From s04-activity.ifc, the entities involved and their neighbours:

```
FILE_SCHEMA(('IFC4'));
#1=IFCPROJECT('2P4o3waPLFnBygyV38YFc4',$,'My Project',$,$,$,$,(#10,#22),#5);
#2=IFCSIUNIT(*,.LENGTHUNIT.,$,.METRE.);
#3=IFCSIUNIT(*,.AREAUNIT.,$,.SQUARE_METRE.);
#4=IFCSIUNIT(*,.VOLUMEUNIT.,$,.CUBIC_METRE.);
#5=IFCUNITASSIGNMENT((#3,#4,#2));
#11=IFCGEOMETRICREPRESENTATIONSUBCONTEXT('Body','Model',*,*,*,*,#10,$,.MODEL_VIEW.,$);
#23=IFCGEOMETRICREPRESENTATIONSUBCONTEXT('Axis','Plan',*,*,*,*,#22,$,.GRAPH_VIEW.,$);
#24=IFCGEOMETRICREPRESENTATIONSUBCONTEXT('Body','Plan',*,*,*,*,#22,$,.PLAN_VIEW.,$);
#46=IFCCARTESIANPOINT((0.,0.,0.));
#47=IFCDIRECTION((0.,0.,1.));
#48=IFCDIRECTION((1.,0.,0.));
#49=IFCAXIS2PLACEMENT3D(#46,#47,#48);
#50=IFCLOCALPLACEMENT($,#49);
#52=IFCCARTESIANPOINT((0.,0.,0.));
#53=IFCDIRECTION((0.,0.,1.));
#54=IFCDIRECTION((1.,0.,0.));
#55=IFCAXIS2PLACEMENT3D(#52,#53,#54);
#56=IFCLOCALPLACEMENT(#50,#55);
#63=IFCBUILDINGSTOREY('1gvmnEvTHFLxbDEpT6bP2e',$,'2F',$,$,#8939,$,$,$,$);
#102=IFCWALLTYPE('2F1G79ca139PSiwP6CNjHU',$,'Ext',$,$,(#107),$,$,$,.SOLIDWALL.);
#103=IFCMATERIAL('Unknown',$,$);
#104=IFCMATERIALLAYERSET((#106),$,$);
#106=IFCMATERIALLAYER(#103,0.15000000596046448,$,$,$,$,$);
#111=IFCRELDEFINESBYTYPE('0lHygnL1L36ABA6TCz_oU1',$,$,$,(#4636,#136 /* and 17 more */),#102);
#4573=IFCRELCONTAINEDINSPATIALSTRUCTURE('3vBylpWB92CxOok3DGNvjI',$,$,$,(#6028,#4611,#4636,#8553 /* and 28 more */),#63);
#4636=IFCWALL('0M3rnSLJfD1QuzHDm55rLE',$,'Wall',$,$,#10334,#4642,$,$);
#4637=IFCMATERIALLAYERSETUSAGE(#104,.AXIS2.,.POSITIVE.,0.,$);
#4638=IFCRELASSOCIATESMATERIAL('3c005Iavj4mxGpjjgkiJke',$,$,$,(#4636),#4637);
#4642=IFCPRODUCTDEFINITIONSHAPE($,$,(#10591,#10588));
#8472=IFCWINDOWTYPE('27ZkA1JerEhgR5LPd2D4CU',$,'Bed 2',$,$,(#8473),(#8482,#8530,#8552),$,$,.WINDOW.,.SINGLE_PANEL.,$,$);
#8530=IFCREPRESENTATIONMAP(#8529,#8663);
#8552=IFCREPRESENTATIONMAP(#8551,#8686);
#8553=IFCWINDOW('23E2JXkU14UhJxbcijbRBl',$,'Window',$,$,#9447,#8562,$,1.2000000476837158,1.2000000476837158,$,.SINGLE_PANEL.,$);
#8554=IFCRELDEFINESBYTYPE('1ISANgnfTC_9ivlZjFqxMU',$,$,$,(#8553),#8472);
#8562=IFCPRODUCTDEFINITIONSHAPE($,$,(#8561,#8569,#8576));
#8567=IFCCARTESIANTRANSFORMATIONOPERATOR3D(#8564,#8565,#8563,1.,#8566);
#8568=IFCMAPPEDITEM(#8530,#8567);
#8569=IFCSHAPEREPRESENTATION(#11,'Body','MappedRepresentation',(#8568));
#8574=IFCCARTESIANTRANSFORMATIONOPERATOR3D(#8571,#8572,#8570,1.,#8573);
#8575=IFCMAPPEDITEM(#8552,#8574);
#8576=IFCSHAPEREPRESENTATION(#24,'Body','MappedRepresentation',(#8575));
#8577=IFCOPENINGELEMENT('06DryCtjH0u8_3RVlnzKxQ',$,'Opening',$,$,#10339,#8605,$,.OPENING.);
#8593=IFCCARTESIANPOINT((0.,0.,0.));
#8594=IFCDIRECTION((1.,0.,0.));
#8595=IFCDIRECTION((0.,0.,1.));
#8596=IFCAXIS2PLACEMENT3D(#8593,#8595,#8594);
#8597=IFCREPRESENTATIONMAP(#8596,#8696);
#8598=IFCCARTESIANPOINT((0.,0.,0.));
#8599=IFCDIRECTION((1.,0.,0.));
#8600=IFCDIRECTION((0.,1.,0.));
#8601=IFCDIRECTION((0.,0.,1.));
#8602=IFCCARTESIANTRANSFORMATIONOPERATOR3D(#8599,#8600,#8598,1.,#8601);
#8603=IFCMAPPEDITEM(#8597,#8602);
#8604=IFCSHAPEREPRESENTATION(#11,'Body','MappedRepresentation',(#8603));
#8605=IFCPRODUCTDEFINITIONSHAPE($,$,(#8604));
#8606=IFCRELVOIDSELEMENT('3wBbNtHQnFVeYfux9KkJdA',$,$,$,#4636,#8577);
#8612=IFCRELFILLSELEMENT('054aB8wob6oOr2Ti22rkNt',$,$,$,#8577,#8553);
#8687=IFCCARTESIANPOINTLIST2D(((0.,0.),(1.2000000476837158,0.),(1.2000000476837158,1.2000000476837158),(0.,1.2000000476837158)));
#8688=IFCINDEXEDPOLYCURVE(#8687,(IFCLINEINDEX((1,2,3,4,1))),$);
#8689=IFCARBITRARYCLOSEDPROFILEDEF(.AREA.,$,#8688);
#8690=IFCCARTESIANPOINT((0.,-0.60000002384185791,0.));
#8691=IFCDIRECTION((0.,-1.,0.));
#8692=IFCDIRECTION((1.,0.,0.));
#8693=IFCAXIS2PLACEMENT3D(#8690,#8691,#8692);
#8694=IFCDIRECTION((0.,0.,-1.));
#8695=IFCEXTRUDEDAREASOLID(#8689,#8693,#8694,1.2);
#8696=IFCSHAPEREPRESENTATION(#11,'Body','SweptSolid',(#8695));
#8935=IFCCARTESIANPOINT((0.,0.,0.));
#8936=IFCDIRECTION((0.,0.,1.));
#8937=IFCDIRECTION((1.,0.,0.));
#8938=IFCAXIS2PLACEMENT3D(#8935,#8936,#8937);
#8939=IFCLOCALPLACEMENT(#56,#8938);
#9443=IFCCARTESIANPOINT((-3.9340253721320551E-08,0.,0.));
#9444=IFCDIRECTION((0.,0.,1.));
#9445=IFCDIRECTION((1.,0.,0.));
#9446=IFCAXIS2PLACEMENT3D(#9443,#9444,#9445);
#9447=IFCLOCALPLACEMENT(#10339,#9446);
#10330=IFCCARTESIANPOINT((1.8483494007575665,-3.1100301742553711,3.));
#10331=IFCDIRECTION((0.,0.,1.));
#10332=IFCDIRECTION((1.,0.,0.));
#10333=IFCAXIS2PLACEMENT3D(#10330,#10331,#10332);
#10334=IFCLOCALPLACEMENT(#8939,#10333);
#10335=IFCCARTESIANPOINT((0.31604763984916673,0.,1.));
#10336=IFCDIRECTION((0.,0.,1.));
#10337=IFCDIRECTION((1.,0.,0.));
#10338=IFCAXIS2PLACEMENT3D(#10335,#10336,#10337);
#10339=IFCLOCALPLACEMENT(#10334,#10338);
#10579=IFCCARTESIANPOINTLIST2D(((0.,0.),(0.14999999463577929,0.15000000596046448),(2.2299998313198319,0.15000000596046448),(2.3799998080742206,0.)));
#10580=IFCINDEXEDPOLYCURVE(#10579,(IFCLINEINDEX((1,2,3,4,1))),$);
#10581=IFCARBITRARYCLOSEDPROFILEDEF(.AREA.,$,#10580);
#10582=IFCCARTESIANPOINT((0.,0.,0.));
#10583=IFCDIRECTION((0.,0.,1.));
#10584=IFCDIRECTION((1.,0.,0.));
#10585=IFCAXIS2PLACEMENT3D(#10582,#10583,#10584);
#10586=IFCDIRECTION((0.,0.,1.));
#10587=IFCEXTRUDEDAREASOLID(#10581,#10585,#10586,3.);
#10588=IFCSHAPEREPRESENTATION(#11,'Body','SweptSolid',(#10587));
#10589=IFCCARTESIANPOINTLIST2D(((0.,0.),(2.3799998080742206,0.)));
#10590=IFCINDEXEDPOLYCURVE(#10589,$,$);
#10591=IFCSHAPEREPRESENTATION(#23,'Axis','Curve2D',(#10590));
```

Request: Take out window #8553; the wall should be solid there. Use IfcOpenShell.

```python
import ifcopenshell
import ifcopenshell.api.feature
import ifcopenshell.api.root
import ifcopenshell.geom
import ifcopenshell.util.shape

model = ifcopenshell.open("s04-activity.ifc")
settings = ifcopenshell.geom.settings()


def volume(element):
    """Net volume in cubic metres, openings subtracted."""
    shape = ifcopenshell.geom.create_shape(settings, element)
    return ifcopenshell.util.shape.get_volume(shape.geometry)


window = model.by_id(8553)
opening = window.FillsVoids[0].RelatingOpeningElement
wall = opening.VoidsElements[0].RelatingBuildingElement
before = volume(wall)

ifcopenshell.api.root.remove_product(model, product=window)
ifcopenshell.api.feature.remove_feature(model, feature=opening)

after = volume(wall)

print(f"wall volume {before:.3f} -> {after:.3f} m3")

model.write("s04-activity-out.ifc")
```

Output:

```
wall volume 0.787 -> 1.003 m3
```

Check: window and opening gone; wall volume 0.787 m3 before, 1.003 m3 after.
